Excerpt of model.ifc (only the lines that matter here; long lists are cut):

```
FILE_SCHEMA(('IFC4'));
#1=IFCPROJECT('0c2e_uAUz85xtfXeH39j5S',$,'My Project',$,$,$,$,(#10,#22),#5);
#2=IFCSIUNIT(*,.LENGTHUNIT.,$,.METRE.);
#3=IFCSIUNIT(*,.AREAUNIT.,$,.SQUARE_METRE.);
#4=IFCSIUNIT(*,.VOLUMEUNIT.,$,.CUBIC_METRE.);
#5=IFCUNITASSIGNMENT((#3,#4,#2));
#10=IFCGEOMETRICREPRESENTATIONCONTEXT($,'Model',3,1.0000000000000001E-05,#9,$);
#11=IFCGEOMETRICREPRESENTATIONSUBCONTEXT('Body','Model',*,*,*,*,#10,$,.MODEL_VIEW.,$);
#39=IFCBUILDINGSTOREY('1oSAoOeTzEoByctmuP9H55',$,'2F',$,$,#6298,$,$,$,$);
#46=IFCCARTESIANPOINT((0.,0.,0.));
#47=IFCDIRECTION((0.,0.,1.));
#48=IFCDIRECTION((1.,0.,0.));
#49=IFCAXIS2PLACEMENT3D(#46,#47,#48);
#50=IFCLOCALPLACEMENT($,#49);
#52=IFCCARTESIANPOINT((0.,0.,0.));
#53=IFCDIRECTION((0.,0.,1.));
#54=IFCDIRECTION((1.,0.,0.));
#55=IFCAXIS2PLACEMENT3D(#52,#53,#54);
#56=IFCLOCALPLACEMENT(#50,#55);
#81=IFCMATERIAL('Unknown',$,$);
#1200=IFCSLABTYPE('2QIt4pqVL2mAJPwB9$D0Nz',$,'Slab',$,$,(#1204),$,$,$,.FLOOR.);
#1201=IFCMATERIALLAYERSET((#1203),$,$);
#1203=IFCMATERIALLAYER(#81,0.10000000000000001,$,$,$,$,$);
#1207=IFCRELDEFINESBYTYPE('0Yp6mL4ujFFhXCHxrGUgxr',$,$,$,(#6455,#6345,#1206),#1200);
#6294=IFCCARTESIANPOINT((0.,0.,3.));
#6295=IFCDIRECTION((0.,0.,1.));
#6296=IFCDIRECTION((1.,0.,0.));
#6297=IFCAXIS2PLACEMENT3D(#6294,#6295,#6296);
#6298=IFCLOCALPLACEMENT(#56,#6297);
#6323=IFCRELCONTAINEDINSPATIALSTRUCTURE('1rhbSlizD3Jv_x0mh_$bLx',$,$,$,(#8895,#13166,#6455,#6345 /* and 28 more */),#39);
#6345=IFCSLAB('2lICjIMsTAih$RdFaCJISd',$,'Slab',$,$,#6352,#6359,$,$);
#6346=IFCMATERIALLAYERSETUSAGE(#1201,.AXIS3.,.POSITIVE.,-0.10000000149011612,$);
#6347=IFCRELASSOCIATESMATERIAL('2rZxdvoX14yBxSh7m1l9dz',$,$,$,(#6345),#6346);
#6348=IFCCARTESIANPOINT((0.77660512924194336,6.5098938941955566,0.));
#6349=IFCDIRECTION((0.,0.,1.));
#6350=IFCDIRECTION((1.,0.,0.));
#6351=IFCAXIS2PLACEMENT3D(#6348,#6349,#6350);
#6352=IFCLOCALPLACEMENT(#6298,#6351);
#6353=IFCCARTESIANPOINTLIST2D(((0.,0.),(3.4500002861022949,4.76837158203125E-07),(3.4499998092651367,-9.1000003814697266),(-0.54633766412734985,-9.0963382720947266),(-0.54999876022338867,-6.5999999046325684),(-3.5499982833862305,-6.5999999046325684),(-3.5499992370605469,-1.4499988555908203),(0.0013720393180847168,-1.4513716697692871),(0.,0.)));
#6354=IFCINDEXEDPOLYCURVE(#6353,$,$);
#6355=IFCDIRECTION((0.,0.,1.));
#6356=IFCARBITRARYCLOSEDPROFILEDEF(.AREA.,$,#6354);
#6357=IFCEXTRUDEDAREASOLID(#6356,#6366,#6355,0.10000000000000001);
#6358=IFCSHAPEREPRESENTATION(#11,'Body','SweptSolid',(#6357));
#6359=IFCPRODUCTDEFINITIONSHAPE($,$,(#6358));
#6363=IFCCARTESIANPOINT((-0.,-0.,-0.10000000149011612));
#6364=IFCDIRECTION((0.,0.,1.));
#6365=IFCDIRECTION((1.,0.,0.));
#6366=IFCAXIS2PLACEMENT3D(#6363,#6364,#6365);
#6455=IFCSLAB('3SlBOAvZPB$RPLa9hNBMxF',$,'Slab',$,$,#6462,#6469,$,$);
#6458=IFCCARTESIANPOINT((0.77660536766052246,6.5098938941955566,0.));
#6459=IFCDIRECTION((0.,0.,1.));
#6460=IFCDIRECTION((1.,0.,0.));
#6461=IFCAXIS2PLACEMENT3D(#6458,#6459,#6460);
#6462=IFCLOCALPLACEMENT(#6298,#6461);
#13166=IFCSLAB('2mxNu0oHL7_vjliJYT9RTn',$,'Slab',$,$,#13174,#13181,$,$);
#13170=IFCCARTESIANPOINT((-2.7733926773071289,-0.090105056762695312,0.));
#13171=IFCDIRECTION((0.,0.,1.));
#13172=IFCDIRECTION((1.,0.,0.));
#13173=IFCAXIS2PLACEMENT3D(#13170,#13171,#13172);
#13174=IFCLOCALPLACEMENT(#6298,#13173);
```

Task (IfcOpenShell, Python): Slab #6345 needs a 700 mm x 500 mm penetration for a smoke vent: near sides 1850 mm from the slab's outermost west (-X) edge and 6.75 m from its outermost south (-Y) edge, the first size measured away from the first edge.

```python
import numpy as np
import ifcopenshell
import ifcopenshell.api.feature
import ifcopenshell.api.geometry
import ifcopenshell.api.root
import ifcopenshell.geom
import ifcopenshell.util.placement
import ifcopenshell.util.representation
import ifcopenshell.util.shape
import ifcopenshell.util.unit

model = ifcopenshell.open("model.ifc")
unit_scale = ifcopenshell.util.unit.calculate_unit_scale(model)
settings = ifcopenshell.geom.settings()


def volume(element):
    """Net volume in cubic metres, openings subtracted."""
    shape = ifcopenshell.geom.create_shape(settings, element)
    return ifcopenshell.util.shape.get_volume(shape.geometry)


slab = model.by_guid("2lICjIMsTAih$RdFaCJISd")
before = volume(slab)

# Extent in the slab's own axes, in metres. The edges named are its -X and -Y sides.
slab_shape = ifcopenshell.geom.create_shape(settings, slab)
vertices = ifcopenshell.util.shape.get_vertices(slab_shape.geometry)
x_min, y_min, bottom = vertices.min(axis=0)
top = vertices[:, 2].max()

opening = ifcopenshell.api.root.create_entity(model, ifc_class="IfcOpeningElement", name="Smoke vent opening", predefined_type="OPENING")
context = ifcopenshell.util.representation.get_context(model, "Model", "Body", "MODEL_VIEW")
width, depth = 0.7, 0.5
outline = [(0.0, 0.0), (width, 0.0), (width, depth), (0.0, depth), (0.0, 0.0)]
# Overshoot both faces by 50 mm so the cut is clean.
shape = ifcopenshell.api.geometry.add_slab_representation(
    model, context=context, depth=top - bottom + 0.1, polyline=outline
)
ifcopenshell.api.geometry.assign_representation(model, product=opening, representation=shape)

matrix = ifcopenshell.util.placement.get_local_placement(slab.ObjectPlacement)
matrix[:, 3] = matrix @ np.append(np.array([x_min + 1.85, y_min + 6.75, bottom - 0.05]) / unit_scale, 1.0)
ifcopenshell.api.geometry.edit_object_placement(model, product=opening, matrix=matrix, is_si=False)
ifcopenshell.api.feature.add_feature(model, feature=opening, element=slab)

after = volume(slab)

print(f"slab volume {before:.3f} -> {after:.3f} m3")

model.write("model-out.ifc")
```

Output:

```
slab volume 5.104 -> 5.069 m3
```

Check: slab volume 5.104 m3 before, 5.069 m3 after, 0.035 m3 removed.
